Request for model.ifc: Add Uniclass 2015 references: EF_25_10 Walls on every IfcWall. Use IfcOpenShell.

First a look at what the model holds.

```python
import ifcopenshell

model = ifcopenshell.open("model.ifc")
print(model.schema)
print("classifications:", [c.Name for c in model.by_type("IfcClassification")])
for ifc_class in ("IfcDoor", "IfcRoof", "IfcStair", "IfcWall", "IfcWindow"):
    print(ifc_class, len(model.by_type(ifc_class)))
```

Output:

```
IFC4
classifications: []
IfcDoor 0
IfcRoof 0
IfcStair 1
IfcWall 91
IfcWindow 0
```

```python
import ifcopenshell
import ifcopenshell.api.classification

model = ifcopenshell.open("model.ifc")

system = ifcopenshell.api.classification.add_classification(model, classification="Uniclass 2015")

codes = {
    "IfcWall": ("EF_25_10", "Walls"),
}
for ifc_class, (code, name) in codes.items():
    products = model.by_type(ifc_class)
    ifcopenshell.api.classification.add_reference(
        model, products=products, classification=system, identification=code, name=name
    )
    print(code, len(products))

model.write("model_v2.ifc")
```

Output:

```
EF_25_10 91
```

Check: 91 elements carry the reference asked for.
